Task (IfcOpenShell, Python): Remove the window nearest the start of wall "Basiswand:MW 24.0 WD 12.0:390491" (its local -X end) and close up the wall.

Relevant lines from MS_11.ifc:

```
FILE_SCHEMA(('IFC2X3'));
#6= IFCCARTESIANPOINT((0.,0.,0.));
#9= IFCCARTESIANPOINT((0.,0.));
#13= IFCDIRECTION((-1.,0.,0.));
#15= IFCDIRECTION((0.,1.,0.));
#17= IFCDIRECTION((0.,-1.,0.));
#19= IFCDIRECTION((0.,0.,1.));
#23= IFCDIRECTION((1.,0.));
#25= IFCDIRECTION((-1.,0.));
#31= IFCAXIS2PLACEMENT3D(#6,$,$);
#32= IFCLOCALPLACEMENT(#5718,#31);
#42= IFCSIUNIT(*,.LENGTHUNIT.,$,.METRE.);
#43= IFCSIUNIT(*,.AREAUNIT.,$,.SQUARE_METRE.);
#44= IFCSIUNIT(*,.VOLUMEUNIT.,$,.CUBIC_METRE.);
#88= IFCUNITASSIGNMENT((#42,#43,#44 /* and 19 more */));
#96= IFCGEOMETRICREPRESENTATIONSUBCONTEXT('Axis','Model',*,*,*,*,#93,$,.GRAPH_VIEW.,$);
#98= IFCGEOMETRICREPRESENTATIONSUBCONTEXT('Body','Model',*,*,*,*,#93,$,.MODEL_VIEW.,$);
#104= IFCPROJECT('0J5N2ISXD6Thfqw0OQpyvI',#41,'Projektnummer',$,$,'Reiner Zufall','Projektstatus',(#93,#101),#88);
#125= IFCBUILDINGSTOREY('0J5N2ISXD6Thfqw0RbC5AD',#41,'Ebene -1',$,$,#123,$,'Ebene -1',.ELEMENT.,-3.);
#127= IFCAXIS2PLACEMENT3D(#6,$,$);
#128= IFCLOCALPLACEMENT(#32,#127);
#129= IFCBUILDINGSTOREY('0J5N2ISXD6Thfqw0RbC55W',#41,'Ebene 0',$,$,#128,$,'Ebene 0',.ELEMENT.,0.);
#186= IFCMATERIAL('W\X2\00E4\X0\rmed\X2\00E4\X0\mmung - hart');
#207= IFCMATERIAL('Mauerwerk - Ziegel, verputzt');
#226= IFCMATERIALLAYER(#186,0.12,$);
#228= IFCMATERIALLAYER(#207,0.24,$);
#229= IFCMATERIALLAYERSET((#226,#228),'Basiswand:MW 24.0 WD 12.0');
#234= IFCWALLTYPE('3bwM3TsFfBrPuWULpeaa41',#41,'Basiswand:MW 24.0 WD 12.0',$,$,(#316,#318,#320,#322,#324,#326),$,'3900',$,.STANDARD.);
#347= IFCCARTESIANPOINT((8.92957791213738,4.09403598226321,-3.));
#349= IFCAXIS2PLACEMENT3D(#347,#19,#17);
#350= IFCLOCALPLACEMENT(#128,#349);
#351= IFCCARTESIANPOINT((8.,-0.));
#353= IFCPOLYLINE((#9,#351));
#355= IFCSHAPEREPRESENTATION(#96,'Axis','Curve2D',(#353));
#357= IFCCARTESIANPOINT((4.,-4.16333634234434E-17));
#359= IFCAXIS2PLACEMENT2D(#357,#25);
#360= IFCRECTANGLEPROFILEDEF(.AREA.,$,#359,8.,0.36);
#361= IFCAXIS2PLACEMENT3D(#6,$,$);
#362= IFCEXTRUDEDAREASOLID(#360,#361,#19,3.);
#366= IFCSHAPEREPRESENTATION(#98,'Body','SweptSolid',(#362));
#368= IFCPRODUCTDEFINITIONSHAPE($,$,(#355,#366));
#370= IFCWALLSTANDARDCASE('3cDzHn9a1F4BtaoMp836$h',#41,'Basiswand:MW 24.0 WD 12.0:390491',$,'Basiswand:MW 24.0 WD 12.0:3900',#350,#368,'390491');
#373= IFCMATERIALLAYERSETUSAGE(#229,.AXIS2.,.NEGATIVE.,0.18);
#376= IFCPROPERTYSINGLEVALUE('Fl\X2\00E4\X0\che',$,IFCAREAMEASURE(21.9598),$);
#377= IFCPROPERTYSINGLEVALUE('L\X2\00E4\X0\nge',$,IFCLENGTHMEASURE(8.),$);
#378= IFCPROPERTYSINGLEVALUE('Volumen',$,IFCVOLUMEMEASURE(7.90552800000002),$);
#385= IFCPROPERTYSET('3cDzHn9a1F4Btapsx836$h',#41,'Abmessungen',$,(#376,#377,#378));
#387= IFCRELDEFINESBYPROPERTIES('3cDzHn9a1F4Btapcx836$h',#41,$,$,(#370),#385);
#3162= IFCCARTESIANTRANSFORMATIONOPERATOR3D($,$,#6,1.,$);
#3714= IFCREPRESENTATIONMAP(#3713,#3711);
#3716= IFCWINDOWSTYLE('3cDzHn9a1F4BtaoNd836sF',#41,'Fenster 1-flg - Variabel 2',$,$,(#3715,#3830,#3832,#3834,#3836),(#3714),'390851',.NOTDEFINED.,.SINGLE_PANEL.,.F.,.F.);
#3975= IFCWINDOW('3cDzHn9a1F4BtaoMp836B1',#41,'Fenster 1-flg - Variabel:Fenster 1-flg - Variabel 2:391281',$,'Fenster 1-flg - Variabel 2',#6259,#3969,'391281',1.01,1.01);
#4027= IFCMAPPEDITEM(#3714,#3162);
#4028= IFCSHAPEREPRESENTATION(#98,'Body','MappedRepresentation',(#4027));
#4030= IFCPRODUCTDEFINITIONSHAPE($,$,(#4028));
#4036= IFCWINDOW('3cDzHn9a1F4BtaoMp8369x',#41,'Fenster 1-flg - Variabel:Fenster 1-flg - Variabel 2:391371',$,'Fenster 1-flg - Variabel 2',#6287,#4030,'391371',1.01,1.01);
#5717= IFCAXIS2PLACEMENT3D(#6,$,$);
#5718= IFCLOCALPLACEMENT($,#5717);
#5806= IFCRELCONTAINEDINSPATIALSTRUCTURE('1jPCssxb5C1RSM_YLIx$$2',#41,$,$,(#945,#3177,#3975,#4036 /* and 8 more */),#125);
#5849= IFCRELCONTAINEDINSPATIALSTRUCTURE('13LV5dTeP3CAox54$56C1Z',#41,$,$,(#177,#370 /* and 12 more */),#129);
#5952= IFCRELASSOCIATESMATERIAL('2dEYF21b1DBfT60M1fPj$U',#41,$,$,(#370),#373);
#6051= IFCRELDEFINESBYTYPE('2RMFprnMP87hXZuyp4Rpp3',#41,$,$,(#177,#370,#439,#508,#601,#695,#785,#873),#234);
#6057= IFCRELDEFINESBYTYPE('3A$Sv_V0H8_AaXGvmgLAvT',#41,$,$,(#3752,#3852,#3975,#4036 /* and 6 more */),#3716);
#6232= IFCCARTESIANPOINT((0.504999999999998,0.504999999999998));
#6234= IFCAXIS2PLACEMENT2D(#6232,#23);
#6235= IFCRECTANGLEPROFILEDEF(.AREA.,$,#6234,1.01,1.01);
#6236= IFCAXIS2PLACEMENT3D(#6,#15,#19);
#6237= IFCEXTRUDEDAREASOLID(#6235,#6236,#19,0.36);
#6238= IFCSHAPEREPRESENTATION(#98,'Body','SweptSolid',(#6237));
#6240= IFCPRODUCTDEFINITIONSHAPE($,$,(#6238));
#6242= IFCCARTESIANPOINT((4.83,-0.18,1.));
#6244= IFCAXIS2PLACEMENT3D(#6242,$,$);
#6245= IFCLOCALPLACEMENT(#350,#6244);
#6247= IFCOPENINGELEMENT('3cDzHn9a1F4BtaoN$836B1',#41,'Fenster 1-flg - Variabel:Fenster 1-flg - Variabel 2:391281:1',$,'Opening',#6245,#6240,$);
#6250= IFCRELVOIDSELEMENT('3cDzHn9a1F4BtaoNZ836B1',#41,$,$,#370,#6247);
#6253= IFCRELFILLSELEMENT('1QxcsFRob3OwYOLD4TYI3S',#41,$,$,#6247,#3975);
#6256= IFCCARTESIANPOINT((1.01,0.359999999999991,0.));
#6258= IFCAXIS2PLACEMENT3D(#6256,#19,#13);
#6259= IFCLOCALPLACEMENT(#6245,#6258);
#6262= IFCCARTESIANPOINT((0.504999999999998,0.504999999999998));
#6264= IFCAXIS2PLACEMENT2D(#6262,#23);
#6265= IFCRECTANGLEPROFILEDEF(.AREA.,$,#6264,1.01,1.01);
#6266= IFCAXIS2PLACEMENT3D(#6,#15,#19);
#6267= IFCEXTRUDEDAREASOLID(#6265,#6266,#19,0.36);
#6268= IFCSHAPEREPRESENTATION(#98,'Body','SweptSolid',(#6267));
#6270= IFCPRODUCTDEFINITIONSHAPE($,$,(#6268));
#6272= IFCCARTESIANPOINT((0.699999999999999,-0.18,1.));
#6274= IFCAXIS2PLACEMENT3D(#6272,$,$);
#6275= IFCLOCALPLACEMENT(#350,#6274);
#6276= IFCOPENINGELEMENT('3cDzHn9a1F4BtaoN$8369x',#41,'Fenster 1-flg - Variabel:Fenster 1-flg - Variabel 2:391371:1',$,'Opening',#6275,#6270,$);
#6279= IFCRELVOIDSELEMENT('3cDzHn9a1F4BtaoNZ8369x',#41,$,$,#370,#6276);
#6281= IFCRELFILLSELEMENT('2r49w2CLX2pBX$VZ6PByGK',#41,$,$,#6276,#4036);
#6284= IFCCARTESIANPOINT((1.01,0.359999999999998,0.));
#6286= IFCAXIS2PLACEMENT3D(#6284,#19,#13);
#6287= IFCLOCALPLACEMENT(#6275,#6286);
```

```python
import ifcopenshell
import ifcopenshell.api.feature
import ifcopenshell.api.pset
import ifcopenshell.api.root
import ifcopenshell.geom
import ifcopenshell.util.element
import ifcopenshell.util.shape
import ifcopenshell.util.unit

model = ifcopenshell.open("MS_11.ifc")
area_scale = ifcopenshell.util.unit.calculate_unit_scale(model, "AREAUNIT")
volume_scale = ifcopenshell.util.unit.calculate_unit_scale(model, "VOLUMEUNIT")
settings = ifcopenshell.geom.settings()


def volume(element):
    """Net volume in cubic metres, openings subtracted."""
    shape = ifcopenshell.geom.create_shape(settings, element)
    return ifcopenshell.util.shape.get_volume(shape.geometry)


window = model.by_guid("3cDzHn9a1F4BtaoMp8369x")
opening = window.FillsVoids[0].RelatingOpeningElement
wall = opening.VoidsElements[0].RelatingBuildingElement
before = volume(wall)

ifcopenshell.api.root.remove_product(model, product=window)
ifcopenshell.api.feature.remove_feature(model, feature=opening)

after = volume(wall)
thickness = 0.36  # wall thickness in metres

# Update the wall's stored quantities.
pset = model.by_id(ifcopenshell.util.element.get_pset(wall, "Abmessungen", should_inherit=False)["id"])
ifcopenshell.api.pset.edit_pset(model, pset=pset, properties={
    "Fläche": model.create_entity("IfcAreaMeasure", after / thickness / area_scale),
    "Volumen": model.create_entity("IfcVolumeMeasure", after / volume_scale),
})

print(f"wall volume {before:.3f} -> {after:.3f} m3")

model.write("MS_11-out.ifc")
```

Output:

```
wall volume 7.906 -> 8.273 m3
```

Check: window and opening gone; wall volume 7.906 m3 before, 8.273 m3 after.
